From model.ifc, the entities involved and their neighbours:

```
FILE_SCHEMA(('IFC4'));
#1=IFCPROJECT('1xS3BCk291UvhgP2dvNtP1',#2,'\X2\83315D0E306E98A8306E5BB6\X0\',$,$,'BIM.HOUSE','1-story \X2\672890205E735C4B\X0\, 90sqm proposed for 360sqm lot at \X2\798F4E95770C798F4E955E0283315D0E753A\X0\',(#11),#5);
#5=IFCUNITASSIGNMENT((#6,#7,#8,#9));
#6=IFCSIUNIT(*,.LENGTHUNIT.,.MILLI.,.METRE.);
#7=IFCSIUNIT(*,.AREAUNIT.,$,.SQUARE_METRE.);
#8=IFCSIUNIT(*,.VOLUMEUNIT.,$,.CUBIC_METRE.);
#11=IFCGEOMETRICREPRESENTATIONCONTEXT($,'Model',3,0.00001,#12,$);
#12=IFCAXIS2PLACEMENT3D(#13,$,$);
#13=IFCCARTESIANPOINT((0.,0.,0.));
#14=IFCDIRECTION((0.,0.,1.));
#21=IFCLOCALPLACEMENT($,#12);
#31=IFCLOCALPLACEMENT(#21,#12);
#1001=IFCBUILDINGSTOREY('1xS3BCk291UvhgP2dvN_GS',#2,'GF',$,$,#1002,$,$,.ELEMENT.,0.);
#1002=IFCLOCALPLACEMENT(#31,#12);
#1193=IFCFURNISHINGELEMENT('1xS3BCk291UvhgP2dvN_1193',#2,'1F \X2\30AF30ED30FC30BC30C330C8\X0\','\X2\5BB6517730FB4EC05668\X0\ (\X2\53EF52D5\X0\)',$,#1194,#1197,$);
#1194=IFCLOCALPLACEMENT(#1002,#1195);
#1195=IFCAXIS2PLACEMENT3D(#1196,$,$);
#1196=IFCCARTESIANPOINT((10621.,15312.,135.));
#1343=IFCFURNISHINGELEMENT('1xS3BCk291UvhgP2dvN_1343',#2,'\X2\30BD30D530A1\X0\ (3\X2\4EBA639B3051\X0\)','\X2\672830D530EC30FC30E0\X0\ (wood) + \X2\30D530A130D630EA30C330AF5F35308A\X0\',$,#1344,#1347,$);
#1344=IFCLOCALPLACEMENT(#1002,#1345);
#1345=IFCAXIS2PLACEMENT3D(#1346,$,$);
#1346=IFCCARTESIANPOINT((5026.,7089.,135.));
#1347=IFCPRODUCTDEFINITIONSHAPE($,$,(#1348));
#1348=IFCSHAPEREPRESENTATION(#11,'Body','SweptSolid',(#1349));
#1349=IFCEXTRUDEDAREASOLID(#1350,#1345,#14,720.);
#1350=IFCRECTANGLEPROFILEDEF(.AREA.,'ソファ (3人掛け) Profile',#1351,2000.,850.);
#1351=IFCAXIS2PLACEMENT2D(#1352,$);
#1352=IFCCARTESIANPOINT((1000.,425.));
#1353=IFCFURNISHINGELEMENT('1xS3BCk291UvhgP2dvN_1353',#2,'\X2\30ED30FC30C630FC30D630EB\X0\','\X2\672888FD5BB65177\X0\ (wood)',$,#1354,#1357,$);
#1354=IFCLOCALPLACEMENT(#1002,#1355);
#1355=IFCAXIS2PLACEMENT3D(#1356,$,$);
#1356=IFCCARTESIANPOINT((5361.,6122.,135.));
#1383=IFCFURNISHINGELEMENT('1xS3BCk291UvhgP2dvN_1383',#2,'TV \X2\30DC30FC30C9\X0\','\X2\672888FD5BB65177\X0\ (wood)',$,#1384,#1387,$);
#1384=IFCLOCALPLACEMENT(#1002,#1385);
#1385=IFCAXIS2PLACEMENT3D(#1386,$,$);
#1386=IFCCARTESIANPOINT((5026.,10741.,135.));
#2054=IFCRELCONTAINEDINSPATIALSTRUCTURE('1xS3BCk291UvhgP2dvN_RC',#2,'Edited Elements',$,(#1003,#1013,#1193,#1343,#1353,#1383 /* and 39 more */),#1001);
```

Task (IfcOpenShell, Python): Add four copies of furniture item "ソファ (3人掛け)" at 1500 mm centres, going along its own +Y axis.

```python
import ifcopenshell
import ifcopenshell.api.geometry
import ifcopenshell.api.root
import ifcopenshell.util.element
import ifcopenshell.util.placement

model = ifcopenshell.open("model.ifc")


def reuse_history(source, copy):
    """copy_class also copies each property set's owner history, people and application; keep the originals."""
    for rel in copy.IsDefinedBy:
        if rel.is_a("IfcRelDefinesByProperties") and (history := rel.RelatingPropertyDefinition.OwnerHistory):
            rel.RelatingPropertyDefinition.OwnerHistory = source.OwnerHistory
            ifcopenshell.util.element.remove_deep2(model, history)


source = model.by_guid("1xS3BCk291UvhgP2dvN_1343")
base = ifcopenshell.util.placement.get_local_placement(source.ObjectPlacement)
step = base[:3, 1] * 1500.0

for i in range(1, 5):
    copy = ifcopenshell.api.root.copy_class(model, product=source)
    copy.Representation = ifcopenshell.util.element.copy_deep(
        model, source.Representation, exclude=["IfcGeometricRepresentationContext", "IfcRepresentationMap"]
    )
    reuse_history(source, copy)
    matrix = base.copy()
    matrix[:3, 3] += i * step
    print("added at", matrix[:3, 3].round(3) + 0.0)
    ifcopenshell.api.geometry.edit_object_placement(model, product=copy, matrix=matrix, is_si=False)

model.write("model_v2.ifc")
```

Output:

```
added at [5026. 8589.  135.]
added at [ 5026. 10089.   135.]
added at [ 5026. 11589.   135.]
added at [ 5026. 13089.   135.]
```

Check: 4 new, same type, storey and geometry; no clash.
